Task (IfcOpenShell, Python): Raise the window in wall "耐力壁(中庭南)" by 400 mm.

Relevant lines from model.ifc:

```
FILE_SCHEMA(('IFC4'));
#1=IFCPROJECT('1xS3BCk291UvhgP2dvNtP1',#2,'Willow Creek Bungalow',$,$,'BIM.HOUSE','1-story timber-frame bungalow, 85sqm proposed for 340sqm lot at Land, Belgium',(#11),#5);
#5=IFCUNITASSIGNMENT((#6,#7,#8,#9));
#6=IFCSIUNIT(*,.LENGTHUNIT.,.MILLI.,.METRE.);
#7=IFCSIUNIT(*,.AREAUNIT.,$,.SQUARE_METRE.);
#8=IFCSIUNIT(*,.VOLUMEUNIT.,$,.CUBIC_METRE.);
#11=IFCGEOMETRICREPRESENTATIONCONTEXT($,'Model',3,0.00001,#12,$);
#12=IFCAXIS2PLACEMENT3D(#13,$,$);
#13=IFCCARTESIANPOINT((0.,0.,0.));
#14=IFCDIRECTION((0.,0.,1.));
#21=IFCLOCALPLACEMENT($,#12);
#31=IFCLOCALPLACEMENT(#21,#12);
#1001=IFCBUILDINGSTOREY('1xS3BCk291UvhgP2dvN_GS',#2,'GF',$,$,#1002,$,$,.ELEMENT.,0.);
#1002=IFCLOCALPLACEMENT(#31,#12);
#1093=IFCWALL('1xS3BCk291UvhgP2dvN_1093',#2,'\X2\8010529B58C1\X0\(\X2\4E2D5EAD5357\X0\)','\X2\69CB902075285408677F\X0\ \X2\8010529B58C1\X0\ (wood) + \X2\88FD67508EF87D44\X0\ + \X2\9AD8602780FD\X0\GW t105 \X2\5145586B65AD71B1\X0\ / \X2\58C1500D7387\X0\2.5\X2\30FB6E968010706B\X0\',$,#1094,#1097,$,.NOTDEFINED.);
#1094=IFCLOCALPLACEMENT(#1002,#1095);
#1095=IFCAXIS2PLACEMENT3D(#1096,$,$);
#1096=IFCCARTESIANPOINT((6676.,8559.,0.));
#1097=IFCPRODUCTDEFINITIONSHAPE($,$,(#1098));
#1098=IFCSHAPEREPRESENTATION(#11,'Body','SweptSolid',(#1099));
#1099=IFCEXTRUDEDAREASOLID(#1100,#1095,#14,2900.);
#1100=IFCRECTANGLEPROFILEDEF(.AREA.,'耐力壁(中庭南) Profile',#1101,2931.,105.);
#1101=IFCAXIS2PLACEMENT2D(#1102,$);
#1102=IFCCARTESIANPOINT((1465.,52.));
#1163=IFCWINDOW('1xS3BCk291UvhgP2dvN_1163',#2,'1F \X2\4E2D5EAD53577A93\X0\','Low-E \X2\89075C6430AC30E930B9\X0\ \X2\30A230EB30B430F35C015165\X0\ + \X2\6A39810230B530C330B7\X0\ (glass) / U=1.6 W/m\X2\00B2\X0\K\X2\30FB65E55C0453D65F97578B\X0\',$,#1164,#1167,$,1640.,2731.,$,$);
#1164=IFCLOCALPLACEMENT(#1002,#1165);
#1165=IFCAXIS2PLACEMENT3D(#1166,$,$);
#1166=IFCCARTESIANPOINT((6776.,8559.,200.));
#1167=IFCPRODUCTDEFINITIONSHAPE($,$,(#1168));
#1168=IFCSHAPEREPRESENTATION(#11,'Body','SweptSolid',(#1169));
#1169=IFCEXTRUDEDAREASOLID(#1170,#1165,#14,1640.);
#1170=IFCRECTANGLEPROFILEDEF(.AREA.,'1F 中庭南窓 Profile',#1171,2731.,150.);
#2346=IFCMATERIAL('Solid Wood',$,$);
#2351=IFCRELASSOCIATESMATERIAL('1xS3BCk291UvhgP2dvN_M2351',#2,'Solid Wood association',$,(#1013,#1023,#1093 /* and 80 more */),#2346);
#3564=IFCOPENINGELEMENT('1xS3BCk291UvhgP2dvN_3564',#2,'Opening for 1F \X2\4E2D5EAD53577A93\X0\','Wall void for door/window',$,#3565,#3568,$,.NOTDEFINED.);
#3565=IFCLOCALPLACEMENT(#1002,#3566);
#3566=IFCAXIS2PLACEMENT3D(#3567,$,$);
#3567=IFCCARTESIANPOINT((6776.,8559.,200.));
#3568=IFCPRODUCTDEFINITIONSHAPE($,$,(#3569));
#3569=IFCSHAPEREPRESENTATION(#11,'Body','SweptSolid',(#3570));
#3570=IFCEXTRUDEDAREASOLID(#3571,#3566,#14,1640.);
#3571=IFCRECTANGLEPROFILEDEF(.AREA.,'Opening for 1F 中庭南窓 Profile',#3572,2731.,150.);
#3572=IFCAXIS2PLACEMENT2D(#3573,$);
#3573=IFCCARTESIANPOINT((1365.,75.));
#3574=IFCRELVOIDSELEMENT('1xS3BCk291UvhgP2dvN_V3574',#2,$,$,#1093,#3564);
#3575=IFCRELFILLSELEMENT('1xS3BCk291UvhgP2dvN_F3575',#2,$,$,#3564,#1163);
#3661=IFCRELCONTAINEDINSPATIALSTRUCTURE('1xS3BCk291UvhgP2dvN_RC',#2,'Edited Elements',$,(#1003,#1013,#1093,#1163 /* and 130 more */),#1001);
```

```python
import numpy as np
import ifcopenshell
import ifcopenshell.api.geometry
import ifcopenshell.util.placement
import ifcopenshell.util.unit

model = ifcopenshell.open("model.ifc")
unit_scale = ifcopenshell.util.unit.calculate_unit_scale(model)

window = model.by_id(1163)
opening = window.FillsVoids[0].RelatingOpeningElement
dz = 400.0

shift = np.array([0.0, 0.0, dz])
# The window is not placed relative to its opening, so move both.
for product in (opening, window):
    matrix = ifcopenshell.util.placement.get_local_placement(product.ObjectPlacement)
    matrix[:3, 3] += shift
    ifcopenshell.api.geometry.edit_object_placement(model, product=product, matrix=matrix, is_si=False)

print(f"moved by {dz * unit_scale:+.3f} m")

model.write("model_rev.ifc")
```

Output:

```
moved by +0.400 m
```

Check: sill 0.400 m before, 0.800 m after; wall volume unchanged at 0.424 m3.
